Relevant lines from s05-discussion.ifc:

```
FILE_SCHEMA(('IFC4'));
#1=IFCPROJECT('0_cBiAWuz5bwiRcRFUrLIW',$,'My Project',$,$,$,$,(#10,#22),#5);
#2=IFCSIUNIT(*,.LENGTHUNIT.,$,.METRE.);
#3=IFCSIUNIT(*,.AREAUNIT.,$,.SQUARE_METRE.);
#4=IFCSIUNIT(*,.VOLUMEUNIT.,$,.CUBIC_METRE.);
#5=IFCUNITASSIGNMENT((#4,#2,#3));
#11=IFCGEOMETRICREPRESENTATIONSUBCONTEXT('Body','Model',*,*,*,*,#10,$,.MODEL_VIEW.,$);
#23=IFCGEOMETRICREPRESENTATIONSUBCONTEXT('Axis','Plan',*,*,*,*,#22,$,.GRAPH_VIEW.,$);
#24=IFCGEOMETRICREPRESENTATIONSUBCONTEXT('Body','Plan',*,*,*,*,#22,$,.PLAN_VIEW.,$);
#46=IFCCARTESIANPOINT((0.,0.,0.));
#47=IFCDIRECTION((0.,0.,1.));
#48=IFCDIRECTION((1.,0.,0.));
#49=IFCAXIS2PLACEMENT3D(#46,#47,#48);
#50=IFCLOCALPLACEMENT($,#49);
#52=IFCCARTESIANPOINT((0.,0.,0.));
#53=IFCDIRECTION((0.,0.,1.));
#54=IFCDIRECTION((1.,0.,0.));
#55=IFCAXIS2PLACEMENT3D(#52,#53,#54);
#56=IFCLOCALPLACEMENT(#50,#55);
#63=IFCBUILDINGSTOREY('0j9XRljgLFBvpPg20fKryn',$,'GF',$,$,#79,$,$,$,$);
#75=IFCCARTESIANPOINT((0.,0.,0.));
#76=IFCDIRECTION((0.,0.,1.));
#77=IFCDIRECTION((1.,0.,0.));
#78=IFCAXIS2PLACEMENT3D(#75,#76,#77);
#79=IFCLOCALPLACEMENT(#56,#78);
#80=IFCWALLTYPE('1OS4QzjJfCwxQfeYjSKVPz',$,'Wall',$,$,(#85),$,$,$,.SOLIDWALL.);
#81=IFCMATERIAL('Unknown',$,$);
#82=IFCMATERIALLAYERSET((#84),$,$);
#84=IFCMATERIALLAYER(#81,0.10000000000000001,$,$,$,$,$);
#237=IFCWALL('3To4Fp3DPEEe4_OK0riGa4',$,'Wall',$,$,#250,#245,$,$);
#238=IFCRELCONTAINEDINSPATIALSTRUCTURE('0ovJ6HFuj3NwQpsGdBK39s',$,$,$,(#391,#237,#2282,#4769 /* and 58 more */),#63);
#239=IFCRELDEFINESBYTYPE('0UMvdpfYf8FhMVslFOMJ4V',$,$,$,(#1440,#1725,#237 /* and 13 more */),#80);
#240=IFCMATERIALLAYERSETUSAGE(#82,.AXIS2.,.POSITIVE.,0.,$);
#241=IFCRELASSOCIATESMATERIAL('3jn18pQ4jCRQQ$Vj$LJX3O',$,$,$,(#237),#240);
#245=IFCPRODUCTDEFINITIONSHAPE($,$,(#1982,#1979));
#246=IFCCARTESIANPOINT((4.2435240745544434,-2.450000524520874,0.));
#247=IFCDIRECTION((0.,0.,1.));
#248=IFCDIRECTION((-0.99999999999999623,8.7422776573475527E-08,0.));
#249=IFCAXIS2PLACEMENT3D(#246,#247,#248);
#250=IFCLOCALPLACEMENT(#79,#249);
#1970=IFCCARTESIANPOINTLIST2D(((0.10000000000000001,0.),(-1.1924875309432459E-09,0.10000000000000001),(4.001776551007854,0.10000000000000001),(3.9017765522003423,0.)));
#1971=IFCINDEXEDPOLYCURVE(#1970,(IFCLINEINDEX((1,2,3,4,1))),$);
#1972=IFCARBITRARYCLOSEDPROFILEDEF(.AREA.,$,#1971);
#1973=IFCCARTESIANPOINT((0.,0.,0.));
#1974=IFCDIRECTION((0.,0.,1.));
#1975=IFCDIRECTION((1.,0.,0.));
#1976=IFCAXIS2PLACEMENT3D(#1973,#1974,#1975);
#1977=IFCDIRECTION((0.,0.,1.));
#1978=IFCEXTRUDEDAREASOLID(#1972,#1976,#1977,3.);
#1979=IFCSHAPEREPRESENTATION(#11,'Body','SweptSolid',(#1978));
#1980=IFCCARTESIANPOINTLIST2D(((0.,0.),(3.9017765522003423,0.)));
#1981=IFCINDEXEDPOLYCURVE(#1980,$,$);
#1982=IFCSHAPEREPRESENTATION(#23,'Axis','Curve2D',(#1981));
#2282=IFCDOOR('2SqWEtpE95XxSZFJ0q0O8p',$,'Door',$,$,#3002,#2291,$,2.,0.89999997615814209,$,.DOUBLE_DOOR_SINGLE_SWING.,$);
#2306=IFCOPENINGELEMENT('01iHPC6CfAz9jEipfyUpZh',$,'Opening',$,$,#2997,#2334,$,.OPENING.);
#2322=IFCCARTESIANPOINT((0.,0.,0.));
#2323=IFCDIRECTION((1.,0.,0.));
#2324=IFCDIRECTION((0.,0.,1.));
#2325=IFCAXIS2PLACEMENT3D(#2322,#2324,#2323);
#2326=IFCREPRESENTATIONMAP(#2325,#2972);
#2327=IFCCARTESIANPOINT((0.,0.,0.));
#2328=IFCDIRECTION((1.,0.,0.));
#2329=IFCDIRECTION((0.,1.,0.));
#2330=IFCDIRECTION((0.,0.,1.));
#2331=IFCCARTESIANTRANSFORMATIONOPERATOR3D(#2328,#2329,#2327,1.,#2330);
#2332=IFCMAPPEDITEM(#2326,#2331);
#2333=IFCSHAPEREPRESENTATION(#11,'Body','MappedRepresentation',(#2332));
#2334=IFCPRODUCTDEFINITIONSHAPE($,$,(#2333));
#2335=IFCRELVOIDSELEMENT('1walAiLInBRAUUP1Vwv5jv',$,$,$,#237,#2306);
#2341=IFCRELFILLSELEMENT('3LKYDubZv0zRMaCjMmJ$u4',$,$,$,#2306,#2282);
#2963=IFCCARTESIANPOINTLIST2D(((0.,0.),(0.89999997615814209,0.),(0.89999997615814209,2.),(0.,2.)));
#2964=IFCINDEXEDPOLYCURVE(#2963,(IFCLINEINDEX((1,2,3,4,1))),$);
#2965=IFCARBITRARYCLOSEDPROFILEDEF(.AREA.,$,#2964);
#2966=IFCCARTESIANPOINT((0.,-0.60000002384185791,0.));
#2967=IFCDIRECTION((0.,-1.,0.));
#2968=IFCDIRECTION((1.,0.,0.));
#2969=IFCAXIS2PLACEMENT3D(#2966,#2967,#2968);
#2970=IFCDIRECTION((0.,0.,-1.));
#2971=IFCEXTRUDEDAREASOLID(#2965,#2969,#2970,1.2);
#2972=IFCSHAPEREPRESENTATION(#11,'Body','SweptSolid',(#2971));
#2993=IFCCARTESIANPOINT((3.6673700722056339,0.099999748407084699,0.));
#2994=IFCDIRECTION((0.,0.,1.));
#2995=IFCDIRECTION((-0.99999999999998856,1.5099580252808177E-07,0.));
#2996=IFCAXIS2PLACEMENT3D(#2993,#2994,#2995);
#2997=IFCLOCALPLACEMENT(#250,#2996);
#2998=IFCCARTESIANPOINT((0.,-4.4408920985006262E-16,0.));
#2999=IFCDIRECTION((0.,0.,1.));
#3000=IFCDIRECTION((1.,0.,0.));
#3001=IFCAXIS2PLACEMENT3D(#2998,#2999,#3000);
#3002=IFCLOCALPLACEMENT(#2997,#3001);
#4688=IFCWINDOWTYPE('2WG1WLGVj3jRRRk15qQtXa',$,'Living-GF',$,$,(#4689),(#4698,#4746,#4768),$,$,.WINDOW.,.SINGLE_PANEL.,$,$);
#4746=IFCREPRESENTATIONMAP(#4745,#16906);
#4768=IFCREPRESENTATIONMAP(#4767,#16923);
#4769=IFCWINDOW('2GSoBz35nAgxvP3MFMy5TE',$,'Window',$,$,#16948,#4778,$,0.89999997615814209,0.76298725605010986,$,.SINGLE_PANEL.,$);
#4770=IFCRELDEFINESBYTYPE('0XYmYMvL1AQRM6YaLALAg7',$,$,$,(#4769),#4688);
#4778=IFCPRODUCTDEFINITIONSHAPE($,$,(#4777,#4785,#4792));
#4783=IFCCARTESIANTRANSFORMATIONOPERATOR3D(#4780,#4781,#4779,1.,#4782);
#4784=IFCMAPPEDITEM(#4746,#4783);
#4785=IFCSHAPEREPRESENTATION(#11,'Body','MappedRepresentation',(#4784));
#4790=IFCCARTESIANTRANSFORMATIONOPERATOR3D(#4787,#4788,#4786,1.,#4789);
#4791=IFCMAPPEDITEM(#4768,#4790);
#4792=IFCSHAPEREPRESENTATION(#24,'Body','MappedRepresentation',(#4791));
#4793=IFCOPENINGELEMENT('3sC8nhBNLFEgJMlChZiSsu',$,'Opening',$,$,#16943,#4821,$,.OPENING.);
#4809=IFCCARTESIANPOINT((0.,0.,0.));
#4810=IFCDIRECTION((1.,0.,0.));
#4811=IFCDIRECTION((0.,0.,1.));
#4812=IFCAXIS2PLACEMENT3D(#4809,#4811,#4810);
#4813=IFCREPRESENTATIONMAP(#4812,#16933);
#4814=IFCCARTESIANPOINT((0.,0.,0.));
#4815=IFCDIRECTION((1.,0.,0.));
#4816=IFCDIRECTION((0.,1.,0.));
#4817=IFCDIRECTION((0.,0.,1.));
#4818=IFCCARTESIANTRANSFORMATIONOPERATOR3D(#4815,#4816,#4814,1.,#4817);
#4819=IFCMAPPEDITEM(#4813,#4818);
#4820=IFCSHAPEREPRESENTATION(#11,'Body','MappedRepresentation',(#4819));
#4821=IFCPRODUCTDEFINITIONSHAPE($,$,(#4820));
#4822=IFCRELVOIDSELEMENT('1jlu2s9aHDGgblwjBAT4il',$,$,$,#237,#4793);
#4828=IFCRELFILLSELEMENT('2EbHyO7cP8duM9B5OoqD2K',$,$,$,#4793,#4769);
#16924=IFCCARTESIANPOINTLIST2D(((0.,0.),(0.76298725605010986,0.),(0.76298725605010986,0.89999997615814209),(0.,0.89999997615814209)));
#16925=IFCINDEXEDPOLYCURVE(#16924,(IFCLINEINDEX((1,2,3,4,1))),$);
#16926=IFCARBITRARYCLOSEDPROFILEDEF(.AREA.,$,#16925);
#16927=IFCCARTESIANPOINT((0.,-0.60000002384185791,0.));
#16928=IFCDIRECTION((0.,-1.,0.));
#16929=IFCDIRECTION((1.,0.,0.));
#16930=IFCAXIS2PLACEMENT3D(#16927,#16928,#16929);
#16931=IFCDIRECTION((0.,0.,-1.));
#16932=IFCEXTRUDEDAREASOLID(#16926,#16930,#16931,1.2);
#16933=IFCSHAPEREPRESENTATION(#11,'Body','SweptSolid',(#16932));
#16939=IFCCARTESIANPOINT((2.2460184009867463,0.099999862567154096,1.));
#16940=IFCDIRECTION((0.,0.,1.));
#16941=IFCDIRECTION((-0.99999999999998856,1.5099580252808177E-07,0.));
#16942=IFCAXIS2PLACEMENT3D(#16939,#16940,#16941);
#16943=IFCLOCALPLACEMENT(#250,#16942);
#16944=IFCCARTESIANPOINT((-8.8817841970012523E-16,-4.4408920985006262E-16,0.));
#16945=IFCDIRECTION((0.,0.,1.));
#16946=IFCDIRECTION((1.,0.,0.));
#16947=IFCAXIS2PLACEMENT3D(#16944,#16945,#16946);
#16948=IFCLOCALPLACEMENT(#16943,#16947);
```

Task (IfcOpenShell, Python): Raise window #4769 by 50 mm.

```python
import numpy as np
import ifcopenshell
import ifcopenshell.api.geometry
import ifcopenshell.util.placement
import ifcopenshell.util.unit

model = ifcopenshell.open("s05-discussion.ifc")
unit_scale = ifcopenshell.util.unit.calculate_unit_scale(model)

window = model.by_id(4769)
opening = window.FillsVoids[0].RelatingOpeningElement
dz = 0.05 / unit_scale

shift = np.array([0.0, 0.0, dz])
# The window is placed relative to its opening, so it follows when the opening moves.
matrix = ifcopenshell.util.placement.get_local_placement(opening.ObjectPlacement)
matrix[:3, 3] += shift
ifcopenshell.api.geometry.edit_object_placement(
    model, product=opening, matrix=matrix, is_si=False, should_transform_children=True
)

print(f"moved by {dz * unit_scale:+.3f} m")

model.write("s05-discussion-out.ifc")
```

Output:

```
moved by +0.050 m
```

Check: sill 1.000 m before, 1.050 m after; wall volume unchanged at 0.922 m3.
